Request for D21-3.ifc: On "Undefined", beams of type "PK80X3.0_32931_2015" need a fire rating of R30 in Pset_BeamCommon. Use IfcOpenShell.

First a look at what the model holds.

```python
import ifcopenshell
import ifcopenshell.util.element

model = ifcopenshell.open("D21-3.ifc")
print(model.schema)
storey = next(s for s in model.by_type("IfcBuildingStorey") if s.Name == "Undefined")
beams = [e for e in ifcopenshell.util.element.get_decomposition(storey) if e.is_a("IfcBeam")]
seen = {}
for e in beams:
    element_type = ifcopenshell.util.element.get_type(e)
    key = (element_type.Name if element_type != e and element_type else None, ifcopenshell.util.element.get_pset(e, "Pset_BeamCommon", "FireRating"))
    seen[key] = seen.get(key, 0) + 1
for (name, value), count in sorted(seen.items(), key=str):
    print(count, "x", name, "|", value)
```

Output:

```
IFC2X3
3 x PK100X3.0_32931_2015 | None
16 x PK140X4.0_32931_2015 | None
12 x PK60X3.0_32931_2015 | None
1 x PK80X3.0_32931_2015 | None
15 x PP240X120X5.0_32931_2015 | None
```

```python
import ifcopenshell
import ifcopenshell.api.pset
import ifcopenshell.util.element

model = ifcopenshell.open("D21-3.ifc")

storey = next(s for s in model.by_type("IfcBuildingStorey") if s.Name == "Undefined")
beams = [e for e in ifcopenshell.util.element.get_decomposition(storey) if e.is_a("IfcBeam")]

count = 0
for e in beams:
    element_type = ifcopenshell.util.element.get_type(e)
    if element_type in (None, e) or element_type.Name != "PK80X3.0_32931_2015":
        continue
    # add_pset returns the element's existing set when there is one.
    pset = ifcopenshell.api.pset.add_pset(model, product=e, name="Pset_BeamCommon")
    ifcopenshell.api.pset.edit_pset(model, pset=pset, properties={"FireRating": "R30"})
    count += 1

print(count, "beams updated")

model.write("D21-3_edited.ifc")
```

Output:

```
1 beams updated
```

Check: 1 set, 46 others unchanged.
